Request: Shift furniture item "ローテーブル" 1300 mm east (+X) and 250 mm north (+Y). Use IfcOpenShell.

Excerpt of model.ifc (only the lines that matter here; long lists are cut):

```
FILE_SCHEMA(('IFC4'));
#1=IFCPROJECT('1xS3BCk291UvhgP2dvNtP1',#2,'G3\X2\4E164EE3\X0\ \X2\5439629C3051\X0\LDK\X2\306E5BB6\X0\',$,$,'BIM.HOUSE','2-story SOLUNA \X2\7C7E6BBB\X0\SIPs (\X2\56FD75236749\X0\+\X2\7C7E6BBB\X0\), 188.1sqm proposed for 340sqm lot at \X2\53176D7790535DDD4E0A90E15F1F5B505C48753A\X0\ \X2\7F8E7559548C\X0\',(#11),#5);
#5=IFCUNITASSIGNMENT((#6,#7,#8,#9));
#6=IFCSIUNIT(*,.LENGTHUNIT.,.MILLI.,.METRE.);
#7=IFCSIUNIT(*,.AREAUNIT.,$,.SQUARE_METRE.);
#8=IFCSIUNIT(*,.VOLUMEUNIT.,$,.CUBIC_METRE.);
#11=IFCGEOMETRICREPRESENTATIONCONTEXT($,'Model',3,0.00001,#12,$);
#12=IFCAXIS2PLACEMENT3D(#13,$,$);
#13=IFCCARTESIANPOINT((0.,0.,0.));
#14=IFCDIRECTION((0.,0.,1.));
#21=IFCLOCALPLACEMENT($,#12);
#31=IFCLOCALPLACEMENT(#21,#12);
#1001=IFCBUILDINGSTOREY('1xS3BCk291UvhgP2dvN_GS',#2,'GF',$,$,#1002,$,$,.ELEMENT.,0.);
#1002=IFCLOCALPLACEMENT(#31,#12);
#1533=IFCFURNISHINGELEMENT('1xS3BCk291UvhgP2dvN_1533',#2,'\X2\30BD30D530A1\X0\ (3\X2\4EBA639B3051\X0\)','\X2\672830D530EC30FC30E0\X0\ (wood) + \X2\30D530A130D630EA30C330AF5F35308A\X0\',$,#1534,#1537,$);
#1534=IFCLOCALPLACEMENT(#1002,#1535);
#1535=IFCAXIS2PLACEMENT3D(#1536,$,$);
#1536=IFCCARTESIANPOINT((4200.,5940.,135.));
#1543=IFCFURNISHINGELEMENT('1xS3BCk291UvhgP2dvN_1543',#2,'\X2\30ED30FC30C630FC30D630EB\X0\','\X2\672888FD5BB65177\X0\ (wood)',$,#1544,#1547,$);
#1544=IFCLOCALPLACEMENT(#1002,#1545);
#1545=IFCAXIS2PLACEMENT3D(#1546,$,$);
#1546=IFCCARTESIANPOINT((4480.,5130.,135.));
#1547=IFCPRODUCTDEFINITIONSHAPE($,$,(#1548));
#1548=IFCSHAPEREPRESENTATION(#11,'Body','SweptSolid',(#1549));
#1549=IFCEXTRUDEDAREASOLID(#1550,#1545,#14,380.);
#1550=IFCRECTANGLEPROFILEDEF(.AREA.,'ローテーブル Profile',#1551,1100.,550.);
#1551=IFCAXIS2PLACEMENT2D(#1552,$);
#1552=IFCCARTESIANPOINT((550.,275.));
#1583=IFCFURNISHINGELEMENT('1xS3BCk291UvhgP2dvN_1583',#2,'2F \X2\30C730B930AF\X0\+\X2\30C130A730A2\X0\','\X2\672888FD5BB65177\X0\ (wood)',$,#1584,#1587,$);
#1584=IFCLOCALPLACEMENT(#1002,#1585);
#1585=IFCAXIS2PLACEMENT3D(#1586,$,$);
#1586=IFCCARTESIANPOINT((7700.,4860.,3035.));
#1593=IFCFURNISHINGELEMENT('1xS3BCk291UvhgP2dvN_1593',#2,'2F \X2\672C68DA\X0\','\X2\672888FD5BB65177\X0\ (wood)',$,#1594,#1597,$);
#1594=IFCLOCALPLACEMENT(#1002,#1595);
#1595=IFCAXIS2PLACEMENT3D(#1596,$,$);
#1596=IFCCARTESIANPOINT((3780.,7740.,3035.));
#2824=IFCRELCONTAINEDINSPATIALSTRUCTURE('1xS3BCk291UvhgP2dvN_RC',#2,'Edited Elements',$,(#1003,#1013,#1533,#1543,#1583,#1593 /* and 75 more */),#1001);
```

```python
import ifcopenshell
import ifcopenshell.api.geometry
import ifcopenshell.util.placement
import ifcopenshell.util.unit

model = ifcopenshell.open("model.ifc")
unit_scale = ifcopenshell.util.unit.calculate_unit_scale(model)

item = model.by_guid("1xS3BCk291UvhgP2dvN_1543")
matrix = ifcopenshell.util.placement.get_local_placement(item.ObjectPlacement)
matrix[0, 3] += 1.3 / unit_scale
matrix[1, 3] += 0.25 / unit_scale
ifcopenshell.api.geometry.edit_object_placement(model, product=item, matrix=matrix, is_si=False)

print(ifcopenshell.util.placement.get_local_placement(item.ObjectPlacement).round(3) + 0.0)

model.write("model_rev.ifc")
```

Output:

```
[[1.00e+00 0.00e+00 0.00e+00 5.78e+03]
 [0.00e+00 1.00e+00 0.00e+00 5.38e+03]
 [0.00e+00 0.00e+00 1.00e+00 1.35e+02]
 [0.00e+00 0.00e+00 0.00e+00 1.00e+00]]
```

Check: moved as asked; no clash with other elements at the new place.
